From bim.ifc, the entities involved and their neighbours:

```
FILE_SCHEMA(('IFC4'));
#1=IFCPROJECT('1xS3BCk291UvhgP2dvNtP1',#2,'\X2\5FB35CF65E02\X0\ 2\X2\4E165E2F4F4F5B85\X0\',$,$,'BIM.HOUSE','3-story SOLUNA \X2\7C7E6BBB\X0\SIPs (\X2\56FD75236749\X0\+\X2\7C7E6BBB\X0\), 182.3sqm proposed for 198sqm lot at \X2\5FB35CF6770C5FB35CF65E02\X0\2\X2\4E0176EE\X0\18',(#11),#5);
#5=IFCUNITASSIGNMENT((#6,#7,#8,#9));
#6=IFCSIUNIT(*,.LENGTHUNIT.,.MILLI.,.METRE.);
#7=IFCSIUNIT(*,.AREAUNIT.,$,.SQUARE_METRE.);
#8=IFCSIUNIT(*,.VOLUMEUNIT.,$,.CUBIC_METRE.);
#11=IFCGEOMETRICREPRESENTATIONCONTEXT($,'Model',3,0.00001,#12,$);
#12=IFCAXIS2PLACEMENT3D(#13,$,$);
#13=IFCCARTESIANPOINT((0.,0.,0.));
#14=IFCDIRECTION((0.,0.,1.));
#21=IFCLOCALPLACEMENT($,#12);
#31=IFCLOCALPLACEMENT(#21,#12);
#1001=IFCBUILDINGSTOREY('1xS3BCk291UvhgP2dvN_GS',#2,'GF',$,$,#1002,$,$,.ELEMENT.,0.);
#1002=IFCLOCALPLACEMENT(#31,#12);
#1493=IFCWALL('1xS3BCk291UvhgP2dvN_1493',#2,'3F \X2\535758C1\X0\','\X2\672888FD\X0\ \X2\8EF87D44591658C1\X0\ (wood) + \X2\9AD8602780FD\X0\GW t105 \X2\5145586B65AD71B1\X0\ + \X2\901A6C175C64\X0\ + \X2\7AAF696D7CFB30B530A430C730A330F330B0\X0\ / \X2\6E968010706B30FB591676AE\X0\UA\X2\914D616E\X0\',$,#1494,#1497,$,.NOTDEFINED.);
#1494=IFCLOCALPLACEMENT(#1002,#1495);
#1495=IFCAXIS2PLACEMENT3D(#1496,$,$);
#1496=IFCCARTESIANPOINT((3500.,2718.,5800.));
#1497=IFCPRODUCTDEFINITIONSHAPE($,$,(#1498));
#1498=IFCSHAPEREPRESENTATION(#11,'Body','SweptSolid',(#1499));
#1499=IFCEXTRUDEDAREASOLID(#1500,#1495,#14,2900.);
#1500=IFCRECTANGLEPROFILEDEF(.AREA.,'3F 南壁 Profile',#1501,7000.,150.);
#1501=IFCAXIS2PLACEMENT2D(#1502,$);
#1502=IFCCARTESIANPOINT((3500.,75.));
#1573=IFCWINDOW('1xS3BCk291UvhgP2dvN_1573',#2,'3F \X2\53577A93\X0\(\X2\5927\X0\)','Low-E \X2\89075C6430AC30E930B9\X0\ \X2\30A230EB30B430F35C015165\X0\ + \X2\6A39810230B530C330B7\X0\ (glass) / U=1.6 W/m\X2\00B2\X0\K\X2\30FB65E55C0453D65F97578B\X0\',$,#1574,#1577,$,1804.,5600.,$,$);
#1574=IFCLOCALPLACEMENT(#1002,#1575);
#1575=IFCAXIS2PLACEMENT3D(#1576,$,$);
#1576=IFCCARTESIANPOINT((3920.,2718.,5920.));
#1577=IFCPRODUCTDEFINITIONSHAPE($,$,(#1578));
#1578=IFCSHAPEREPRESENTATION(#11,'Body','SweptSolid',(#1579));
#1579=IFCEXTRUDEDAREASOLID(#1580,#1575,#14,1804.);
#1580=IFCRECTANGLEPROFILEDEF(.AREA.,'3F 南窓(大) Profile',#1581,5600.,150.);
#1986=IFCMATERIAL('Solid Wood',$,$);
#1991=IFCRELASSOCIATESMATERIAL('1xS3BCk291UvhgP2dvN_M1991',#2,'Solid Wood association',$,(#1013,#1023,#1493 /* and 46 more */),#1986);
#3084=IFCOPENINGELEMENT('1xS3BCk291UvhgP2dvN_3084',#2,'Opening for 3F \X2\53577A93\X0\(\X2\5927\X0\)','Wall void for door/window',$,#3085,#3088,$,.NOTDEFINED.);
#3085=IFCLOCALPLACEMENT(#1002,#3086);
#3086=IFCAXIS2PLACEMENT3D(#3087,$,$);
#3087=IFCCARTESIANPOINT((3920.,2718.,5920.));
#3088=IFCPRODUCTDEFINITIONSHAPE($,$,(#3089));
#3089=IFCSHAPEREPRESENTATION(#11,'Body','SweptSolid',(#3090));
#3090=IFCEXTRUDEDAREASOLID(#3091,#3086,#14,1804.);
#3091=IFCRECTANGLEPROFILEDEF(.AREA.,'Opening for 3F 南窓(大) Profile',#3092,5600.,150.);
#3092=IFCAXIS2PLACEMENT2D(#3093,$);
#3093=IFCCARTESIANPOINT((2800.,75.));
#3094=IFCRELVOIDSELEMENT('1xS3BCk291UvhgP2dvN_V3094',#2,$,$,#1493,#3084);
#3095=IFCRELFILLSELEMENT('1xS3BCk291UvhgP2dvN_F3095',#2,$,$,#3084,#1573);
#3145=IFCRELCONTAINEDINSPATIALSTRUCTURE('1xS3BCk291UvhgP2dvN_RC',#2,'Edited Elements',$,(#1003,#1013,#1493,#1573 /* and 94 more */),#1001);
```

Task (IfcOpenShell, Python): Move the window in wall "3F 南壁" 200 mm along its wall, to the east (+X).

```python
import ifcopenshell
import ifcopenshell.api.geometry
import ifcopenshell.util.placement
import ifcopenshell.util.unit

model = ifcopenshell.open("bim.ifc")
unit_scale = ifcopenshell.util.unit.calculate_unit_scale(model)

window = model.by_guid("1xS3BCk291UvhgP2dvN_1573")
opening = window.FillsVoids[0].RelatingOpeningElement
wall = opening.VoidsElements[0].RelatingBuildingElement

wall_matrix = ifcopenshell.util.placement.get_local_placement(wall.ObjectPlacement)
shift = wall_matrix[:3, 0] * 0.2 / unit_scale
before = ifcopenshell.util.placement.get_local_placement(window.ObjectPlacement)[:3, 3].copy()

# The window is not placed relative to its opening, so move both.
for product in (opening, window):
    matrix = ifcopenshell.util.placement.get_local_placement(product.ObjectPlacement)
    matrix[:3, 3] += shift
    ifcopenshell.api.geometry.edit_object_placement(model, product=product, matrix=matrix, is_si=False)

after = ifcopenshell.util.placement.get_local_placement(window.ObjectPlacement)[:3, 3]
print("window moved by", (after - before).round(3) + 0.0)

model.write("bim-out.ifc")
```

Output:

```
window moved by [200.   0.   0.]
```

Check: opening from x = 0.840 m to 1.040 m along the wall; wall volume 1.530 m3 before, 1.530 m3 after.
